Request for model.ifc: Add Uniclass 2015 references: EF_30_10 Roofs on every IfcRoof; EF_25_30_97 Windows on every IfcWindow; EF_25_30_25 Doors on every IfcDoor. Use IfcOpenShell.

First a look at what the model holds.

```python
import ifcopenshell

model = ifcopenshell.open("model.ifc")
print(model.schema)
print("classifications:", [c.Name for c in model.by_type("IfcClassification")])
for ifc_class in ("IfcDoor", "IfcRoof", "IfcStair", "IfcWall", "IfcWindow"):
    print(ifc_class, len(model.by_type(ifc_class)))
```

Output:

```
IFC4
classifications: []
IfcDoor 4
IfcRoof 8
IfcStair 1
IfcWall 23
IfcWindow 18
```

```python
import ifcopenshell
import ifcopenshell.api.classification

model = ifcopenshell.open("model.ifc")

system = ifcopenshell.api.classification.add_classification(model, classification="Uniclass 2015")

codes = {
    "IfcRoof": ("EF_30_10", "Roofs"),
    "IfcWindow": ("EF_25_30_97", "Windows"),
    "IfcDoor": ("EF_25_30_25", "Doors"),
}
for ifc_class, (code, name) in codes.items():
    products = model.by_type(ifc_class)
    ifcopenshell.api.classification.add_reference(
        model, products=products, classification=system, identification=code, name=name
    )
    print(code, len(products))

model.write("model_updated.ifc")
```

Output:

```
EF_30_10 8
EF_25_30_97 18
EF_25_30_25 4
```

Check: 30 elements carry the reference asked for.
